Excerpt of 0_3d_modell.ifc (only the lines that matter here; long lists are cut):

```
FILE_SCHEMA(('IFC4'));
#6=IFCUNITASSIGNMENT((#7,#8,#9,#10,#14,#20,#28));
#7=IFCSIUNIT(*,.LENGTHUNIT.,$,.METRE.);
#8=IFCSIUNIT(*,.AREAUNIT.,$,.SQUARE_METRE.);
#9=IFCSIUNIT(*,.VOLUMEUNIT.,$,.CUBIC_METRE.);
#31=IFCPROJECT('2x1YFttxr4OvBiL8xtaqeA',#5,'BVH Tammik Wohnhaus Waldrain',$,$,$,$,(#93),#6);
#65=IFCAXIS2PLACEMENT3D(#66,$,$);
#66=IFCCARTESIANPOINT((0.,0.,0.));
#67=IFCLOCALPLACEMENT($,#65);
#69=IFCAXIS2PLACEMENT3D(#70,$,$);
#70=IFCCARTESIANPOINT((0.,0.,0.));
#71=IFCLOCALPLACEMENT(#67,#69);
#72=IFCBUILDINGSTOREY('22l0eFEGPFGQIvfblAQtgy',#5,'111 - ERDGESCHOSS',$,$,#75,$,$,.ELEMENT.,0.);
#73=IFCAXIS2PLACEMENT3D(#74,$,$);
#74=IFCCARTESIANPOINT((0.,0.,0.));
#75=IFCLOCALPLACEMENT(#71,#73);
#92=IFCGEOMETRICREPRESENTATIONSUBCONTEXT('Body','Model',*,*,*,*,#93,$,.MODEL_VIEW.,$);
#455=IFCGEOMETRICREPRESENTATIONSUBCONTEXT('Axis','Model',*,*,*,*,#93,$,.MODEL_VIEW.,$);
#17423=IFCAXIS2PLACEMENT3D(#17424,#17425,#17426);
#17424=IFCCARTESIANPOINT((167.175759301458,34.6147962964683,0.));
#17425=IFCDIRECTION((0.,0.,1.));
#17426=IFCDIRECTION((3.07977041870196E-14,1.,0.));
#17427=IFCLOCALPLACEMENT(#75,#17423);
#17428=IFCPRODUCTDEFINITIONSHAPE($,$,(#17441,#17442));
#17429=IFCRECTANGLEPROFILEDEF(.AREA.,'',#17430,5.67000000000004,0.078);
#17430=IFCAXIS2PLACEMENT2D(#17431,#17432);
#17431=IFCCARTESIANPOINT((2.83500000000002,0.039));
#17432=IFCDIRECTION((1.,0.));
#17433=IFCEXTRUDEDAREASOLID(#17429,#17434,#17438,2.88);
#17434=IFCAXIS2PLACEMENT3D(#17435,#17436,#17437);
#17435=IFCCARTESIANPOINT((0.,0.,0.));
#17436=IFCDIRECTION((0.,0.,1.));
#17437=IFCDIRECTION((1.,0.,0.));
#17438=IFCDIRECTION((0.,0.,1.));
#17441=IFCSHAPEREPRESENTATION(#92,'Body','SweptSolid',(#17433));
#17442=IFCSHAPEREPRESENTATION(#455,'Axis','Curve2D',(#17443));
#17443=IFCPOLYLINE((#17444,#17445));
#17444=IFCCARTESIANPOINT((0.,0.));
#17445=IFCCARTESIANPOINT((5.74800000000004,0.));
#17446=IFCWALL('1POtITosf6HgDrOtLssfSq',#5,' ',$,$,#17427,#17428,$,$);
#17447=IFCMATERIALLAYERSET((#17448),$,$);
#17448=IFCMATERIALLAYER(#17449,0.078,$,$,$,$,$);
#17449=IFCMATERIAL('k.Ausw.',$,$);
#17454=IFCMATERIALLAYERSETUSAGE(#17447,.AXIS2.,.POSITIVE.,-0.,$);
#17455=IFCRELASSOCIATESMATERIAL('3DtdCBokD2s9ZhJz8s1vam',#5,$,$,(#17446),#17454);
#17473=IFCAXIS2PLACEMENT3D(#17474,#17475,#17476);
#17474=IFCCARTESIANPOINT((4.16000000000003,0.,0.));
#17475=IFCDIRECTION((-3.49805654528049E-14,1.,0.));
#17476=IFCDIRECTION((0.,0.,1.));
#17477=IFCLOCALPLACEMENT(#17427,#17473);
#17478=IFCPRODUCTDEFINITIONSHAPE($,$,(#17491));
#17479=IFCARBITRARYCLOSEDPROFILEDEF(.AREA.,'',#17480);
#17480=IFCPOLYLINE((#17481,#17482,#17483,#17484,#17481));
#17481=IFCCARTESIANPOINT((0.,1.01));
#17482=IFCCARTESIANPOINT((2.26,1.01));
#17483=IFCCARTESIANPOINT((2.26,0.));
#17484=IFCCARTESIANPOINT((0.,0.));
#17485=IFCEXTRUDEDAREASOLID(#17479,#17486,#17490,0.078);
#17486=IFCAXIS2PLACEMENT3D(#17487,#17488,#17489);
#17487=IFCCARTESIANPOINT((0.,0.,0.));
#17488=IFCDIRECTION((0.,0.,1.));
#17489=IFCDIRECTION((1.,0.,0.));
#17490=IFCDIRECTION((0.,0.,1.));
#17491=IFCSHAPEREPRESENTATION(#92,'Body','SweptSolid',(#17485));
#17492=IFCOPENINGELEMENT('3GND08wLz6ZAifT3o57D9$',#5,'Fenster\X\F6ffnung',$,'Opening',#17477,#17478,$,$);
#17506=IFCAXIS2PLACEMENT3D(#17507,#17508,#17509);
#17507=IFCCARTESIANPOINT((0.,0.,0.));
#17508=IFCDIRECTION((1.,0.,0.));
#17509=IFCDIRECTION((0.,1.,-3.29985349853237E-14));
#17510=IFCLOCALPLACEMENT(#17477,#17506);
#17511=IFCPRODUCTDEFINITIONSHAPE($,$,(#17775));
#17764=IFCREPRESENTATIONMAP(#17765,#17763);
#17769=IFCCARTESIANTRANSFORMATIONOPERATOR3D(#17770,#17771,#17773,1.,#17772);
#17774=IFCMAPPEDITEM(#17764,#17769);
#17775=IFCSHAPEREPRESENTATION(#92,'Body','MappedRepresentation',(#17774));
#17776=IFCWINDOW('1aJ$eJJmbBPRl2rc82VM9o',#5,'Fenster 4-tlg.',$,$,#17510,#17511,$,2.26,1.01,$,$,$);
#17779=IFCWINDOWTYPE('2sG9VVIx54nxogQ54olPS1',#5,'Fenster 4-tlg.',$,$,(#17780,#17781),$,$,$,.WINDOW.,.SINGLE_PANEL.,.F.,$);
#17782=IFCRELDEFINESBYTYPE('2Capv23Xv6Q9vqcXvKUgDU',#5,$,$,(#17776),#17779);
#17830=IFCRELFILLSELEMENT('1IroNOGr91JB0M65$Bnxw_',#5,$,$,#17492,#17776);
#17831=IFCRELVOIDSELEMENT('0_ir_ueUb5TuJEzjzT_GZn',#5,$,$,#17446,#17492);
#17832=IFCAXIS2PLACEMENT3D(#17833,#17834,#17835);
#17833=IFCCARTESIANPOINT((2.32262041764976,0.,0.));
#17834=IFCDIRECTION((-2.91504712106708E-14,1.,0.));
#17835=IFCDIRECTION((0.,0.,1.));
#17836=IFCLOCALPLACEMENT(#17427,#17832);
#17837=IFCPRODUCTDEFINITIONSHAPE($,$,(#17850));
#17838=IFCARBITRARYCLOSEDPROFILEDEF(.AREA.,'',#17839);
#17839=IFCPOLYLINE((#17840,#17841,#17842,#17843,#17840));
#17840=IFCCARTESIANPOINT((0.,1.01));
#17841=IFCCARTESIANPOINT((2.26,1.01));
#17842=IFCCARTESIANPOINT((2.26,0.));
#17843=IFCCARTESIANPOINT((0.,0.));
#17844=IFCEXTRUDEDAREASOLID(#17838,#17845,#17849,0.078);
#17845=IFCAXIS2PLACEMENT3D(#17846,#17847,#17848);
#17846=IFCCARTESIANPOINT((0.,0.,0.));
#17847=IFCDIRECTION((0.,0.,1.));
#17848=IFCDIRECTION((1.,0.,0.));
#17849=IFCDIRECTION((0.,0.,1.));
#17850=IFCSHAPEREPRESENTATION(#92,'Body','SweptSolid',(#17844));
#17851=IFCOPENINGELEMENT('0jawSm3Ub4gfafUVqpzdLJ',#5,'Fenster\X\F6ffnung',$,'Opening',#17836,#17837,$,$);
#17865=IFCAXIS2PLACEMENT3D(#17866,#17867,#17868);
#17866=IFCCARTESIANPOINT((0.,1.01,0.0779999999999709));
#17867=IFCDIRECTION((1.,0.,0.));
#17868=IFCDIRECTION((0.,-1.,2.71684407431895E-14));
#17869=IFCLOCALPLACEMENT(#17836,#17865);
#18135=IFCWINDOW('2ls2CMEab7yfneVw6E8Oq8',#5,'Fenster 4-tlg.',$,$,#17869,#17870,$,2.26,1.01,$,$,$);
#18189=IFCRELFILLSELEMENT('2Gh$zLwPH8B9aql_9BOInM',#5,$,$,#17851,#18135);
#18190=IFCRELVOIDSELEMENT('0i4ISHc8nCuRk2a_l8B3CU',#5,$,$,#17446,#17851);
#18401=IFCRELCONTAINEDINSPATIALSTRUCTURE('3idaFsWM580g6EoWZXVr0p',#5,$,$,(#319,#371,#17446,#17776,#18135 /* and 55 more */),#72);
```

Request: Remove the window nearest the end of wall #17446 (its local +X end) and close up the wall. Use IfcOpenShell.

```python
import ifcopenshell
import ifcopenshell.api.feature
import ifcopenshell.api.root
import ifcopenshell.geom
import ifcopenshell.util.shape

model = ifcopenshell.open("0_3d_modell.ifc")
settings = ifcopenshell.geom.settings()


def volume(element):
    """Net volume in cubic metres, openings subtracted."""
    shape = ifcopenshell.geom.create_shape(settings, element)
    return ifcopenshell.util.shape.get_volume(shape.geometry)


window = model.by_id(17776)
opening = window.FillsVoids[0].RelatingOpeningElement
wall = opening.VoidsElements[0].RelatingBuildingElement
before = volume(wall)

ifcopenshell.api.root.remove_product(model, product=window)
ifcopenshell.api.feature.remove_feature(model, feature=opening)

after = volume(wall)

print(f"wall volume {before:.3f} -> {after:.3f} m3")

model.write("0_3d_modell_rev.ifc")
```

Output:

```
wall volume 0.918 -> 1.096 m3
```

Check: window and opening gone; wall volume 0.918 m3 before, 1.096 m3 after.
